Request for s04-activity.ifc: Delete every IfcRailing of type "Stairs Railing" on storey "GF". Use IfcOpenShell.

First a look at what the model holds.

```python
import ifcopenshell
import ifcopenshell.util.element

model = ifcopenshell.open("s04-activity.ifc")
print(model.schema)
storey = next(s for s in model.by_type("IfcBuildingStorey") if s.Name == "GF")
railings = [e for e in ifcopenshell.util.element.get_decomposition(storey) if e.is_a("IfcRailing")]
seen = {}
for e in railings:
    element_type = ifcopenshell.util.element.get_type(e)
    name = element_type.Name if element_type not in (None, e) else None
    seen[name] = seen.get(name, 0) + 1
for name, count in sorted(seen.items(), key=str):
    print(count, "x", name)
```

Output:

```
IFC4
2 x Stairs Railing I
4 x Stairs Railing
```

```python
import ifcopenshell
import ifcopenshell.api.root
import ifcopenshell.util.element

model = ifcopenshell.open("s04-activity.ifc")

storey = next(s for s in model.by_type("IfcBuildingStorey") if s.Name == "GF")
railings = [e for e in ifcopenshell.util.element.get_decomposition(storey) if e.is_a("IfcRailing")]
targets = [e for e in railings if (t := ifcopenshell.util.element.get_type(e)) not in (None, e) and t.Name == "Stairs Railing"]

for e in targets:
    ifcopenshell.api.root.remove_product(model, product=e)
print(len(targets), "removed")

model.write("s04-activity_updated.ifc")
```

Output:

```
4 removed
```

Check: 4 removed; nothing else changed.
